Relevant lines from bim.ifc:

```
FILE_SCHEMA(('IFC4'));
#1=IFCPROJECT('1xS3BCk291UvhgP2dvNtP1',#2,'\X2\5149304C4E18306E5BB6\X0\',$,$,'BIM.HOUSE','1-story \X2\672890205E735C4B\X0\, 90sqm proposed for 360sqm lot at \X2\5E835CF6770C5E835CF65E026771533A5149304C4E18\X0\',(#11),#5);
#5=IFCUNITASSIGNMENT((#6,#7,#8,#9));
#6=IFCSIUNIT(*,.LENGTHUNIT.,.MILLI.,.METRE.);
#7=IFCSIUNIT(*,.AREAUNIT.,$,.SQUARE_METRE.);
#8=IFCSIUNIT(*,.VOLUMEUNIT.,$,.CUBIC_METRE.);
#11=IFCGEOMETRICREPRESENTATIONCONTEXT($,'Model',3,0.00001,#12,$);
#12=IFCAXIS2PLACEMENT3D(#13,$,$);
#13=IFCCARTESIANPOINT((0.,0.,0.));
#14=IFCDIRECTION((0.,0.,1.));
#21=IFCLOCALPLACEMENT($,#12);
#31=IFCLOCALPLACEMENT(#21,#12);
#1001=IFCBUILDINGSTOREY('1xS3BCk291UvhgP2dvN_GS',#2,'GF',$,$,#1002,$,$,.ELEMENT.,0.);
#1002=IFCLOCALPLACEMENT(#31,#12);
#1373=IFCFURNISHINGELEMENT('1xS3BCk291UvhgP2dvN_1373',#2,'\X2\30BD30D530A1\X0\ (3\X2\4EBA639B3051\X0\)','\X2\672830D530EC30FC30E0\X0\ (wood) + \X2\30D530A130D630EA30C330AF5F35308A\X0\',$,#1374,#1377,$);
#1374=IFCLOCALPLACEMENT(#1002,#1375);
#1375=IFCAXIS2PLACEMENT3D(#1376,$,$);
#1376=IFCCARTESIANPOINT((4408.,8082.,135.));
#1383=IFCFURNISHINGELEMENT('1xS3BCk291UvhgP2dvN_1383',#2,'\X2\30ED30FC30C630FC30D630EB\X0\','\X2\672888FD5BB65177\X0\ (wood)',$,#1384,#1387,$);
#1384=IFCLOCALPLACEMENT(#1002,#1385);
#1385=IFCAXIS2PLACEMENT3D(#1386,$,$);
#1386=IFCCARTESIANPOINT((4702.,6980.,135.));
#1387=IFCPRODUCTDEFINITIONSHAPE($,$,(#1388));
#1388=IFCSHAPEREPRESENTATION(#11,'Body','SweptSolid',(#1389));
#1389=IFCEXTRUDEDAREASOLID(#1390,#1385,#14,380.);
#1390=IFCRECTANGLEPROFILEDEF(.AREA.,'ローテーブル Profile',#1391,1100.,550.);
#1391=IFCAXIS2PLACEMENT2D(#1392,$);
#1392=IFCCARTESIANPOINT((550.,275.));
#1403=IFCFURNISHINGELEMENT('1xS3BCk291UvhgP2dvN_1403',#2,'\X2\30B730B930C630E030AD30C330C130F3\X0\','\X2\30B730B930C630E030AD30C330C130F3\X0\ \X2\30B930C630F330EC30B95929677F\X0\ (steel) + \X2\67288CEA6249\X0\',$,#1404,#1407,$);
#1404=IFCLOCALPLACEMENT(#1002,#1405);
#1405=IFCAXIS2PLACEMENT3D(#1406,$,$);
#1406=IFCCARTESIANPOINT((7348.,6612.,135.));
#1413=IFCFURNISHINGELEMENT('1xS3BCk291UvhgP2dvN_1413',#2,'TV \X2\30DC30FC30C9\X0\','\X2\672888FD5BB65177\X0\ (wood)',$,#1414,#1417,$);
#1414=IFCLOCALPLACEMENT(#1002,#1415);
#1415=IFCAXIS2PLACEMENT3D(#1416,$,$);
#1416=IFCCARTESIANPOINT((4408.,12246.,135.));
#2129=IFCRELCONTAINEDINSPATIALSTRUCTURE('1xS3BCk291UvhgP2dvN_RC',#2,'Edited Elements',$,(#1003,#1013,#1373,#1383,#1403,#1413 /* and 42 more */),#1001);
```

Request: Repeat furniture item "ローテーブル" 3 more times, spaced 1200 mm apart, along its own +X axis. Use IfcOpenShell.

```python
import ifcopenshell
import ifcopenshell.api.geometry
import ifcopenshell.api.root
import ifcopenshell.util.element
import ifcopenshell.util.placement
import ifcopenshell.util.unit

model = ifcopenshell.open("bim.ifc")
unit_scale = ifcopenshell.util.unit.calculate_unit_scale(model)


def reuse_history(source, copy):
    """copy_class also copies each property set's owner history, people and application; keep the originals."""
    for rel in copy.IsDefinedBy:
        if rel.is_a("IfcRelDefinesByProperties") and (history := rel.RelatingPropertyDefinition.OwnerHistory):
            rel.RelatingPropertyDefinition.OwnerHistory = source.OwnerHistory
            ifcopenshell.util.element.remove_deep2(model, history)


source = model.by_guid("1xS3BCk291UvhgP2dvN_1383")
base = ifcopenshell.util.placement.get_local_placement(source.ObjectPlacement)
step = base[:3, 0] * 1.2 / unit_scale

for i in range(1, 4):
    copy = ifcopenshell.api.root.copy_class(model, product=source)
    copy.Representation = ifcopenshell.util.element.copy_deep(
        model, source.Representation, exclude=["IfcGeometricRepresentationContext", "IfcRepresentationMap"]
    )
    reuse_history(source, copy)
    matrix = base.copy()
    matrix[:3, 3] += i * step
    print("added at", matrix[:3, 3].round(3) + 0.0)
    ifcopenshell.api.geometry.edit_object_placement(model, product=copy, matrix=matrix, is_si=False)

model.write("bim-out.ifc")
```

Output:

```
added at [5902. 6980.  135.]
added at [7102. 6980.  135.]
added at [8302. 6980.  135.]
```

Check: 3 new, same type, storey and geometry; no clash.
